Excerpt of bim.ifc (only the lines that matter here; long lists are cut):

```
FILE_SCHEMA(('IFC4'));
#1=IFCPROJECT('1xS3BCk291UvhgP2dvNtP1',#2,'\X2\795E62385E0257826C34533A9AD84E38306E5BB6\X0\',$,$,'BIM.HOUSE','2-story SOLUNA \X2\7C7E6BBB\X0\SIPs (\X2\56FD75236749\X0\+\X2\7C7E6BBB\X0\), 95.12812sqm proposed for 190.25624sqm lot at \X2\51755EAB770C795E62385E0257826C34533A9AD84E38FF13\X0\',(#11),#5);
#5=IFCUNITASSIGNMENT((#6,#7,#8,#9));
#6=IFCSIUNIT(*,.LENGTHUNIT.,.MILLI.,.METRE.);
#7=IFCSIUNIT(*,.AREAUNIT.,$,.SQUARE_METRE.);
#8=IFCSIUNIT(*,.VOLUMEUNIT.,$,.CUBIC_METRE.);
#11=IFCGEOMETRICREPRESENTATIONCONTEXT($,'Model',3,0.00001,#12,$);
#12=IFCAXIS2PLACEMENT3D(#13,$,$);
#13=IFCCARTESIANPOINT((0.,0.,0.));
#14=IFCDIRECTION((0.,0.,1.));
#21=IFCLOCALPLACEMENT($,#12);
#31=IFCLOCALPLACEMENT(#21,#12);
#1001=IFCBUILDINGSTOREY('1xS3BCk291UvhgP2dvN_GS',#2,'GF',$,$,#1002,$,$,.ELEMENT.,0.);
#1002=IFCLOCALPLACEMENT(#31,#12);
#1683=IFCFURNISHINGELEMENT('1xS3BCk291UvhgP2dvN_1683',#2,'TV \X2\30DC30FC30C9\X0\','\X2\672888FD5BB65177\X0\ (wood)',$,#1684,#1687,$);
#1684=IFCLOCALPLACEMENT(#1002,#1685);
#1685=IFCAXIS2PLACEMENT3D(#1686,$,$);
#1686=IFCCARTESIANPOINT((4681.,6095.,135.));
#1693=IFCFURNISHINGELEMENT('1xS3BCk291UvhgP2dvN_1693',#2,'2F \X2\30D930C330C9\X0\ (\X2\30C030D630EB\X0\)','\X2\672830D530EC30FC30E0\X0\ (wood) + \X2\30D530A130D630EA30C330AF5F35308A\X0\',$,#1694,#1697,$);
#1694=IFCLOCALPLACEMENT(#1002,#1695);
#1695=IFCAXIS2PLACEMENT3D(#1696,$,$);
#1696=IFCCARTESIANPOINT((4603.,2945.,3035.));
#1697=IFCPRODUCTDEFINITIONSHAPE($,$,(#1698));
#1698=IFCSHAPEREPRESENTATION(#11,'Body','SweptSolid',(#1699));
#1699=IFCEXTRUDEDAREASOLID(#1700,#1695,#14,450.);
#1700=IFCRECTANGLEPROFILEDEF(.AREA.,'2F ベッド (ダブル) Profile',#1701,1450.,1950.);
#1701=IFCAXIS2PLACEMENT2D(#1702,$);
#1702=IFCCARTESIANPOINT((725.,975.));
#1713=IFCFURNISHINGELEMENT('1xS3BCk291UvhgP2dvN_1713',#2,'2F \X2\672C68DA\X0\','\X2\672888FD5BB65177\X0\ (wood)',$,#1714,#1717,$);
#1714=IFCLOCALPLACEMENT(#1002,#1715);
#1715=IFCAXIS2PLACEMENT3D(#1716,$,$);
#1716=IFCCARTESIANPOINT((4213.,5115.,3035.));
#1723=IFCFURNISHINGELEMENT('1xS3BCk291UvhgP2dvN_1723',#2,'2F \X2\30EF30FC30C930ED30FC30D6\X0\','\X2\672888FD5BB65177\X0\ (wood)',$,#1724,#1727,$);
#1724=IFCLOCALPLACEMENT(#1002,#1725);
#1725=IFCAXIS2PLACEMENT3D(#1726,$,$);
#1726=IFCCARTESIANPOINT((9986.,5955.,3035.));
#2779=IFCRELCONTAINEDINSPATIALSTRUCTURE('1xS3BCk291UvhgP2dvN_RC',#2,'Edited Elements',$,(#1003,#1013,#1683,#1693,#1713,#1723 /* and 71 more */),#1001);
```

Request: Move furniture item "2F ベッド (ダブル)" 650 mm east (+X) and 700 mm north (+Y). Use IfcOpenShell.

```python
import ifcopenshell
import ifcopenshell.api.geometry
import ifcopenshell.util.placement

model = ifcopenshell.open("bim.ifc")

item = model.by_guid("1xS3BCk291UvhgP2dvN_1693")
matrix = ifcopenshell.util.placement.get_local_placement(item.ObjectPlacement)
matrix[0, 3] += 650.0
matrix[1, 3] += 700.0
ifcopenshell.api.geometry.edit_object_placement(model, product=item, matrix=matrix, is_si=False)

print(ifcopenshell.util.placement.get_local_placement(item.ObjectPlacement).round(3) + 0.0)

model.write("bim_edited.ifc")
```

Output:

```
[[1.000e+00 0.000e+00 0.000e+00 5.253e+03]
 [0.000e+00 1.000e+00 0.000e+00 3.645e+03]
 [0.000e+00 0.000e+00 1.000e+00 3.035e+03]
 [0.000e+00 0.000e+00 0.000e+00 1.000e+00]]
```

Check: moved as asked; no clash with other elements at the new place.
